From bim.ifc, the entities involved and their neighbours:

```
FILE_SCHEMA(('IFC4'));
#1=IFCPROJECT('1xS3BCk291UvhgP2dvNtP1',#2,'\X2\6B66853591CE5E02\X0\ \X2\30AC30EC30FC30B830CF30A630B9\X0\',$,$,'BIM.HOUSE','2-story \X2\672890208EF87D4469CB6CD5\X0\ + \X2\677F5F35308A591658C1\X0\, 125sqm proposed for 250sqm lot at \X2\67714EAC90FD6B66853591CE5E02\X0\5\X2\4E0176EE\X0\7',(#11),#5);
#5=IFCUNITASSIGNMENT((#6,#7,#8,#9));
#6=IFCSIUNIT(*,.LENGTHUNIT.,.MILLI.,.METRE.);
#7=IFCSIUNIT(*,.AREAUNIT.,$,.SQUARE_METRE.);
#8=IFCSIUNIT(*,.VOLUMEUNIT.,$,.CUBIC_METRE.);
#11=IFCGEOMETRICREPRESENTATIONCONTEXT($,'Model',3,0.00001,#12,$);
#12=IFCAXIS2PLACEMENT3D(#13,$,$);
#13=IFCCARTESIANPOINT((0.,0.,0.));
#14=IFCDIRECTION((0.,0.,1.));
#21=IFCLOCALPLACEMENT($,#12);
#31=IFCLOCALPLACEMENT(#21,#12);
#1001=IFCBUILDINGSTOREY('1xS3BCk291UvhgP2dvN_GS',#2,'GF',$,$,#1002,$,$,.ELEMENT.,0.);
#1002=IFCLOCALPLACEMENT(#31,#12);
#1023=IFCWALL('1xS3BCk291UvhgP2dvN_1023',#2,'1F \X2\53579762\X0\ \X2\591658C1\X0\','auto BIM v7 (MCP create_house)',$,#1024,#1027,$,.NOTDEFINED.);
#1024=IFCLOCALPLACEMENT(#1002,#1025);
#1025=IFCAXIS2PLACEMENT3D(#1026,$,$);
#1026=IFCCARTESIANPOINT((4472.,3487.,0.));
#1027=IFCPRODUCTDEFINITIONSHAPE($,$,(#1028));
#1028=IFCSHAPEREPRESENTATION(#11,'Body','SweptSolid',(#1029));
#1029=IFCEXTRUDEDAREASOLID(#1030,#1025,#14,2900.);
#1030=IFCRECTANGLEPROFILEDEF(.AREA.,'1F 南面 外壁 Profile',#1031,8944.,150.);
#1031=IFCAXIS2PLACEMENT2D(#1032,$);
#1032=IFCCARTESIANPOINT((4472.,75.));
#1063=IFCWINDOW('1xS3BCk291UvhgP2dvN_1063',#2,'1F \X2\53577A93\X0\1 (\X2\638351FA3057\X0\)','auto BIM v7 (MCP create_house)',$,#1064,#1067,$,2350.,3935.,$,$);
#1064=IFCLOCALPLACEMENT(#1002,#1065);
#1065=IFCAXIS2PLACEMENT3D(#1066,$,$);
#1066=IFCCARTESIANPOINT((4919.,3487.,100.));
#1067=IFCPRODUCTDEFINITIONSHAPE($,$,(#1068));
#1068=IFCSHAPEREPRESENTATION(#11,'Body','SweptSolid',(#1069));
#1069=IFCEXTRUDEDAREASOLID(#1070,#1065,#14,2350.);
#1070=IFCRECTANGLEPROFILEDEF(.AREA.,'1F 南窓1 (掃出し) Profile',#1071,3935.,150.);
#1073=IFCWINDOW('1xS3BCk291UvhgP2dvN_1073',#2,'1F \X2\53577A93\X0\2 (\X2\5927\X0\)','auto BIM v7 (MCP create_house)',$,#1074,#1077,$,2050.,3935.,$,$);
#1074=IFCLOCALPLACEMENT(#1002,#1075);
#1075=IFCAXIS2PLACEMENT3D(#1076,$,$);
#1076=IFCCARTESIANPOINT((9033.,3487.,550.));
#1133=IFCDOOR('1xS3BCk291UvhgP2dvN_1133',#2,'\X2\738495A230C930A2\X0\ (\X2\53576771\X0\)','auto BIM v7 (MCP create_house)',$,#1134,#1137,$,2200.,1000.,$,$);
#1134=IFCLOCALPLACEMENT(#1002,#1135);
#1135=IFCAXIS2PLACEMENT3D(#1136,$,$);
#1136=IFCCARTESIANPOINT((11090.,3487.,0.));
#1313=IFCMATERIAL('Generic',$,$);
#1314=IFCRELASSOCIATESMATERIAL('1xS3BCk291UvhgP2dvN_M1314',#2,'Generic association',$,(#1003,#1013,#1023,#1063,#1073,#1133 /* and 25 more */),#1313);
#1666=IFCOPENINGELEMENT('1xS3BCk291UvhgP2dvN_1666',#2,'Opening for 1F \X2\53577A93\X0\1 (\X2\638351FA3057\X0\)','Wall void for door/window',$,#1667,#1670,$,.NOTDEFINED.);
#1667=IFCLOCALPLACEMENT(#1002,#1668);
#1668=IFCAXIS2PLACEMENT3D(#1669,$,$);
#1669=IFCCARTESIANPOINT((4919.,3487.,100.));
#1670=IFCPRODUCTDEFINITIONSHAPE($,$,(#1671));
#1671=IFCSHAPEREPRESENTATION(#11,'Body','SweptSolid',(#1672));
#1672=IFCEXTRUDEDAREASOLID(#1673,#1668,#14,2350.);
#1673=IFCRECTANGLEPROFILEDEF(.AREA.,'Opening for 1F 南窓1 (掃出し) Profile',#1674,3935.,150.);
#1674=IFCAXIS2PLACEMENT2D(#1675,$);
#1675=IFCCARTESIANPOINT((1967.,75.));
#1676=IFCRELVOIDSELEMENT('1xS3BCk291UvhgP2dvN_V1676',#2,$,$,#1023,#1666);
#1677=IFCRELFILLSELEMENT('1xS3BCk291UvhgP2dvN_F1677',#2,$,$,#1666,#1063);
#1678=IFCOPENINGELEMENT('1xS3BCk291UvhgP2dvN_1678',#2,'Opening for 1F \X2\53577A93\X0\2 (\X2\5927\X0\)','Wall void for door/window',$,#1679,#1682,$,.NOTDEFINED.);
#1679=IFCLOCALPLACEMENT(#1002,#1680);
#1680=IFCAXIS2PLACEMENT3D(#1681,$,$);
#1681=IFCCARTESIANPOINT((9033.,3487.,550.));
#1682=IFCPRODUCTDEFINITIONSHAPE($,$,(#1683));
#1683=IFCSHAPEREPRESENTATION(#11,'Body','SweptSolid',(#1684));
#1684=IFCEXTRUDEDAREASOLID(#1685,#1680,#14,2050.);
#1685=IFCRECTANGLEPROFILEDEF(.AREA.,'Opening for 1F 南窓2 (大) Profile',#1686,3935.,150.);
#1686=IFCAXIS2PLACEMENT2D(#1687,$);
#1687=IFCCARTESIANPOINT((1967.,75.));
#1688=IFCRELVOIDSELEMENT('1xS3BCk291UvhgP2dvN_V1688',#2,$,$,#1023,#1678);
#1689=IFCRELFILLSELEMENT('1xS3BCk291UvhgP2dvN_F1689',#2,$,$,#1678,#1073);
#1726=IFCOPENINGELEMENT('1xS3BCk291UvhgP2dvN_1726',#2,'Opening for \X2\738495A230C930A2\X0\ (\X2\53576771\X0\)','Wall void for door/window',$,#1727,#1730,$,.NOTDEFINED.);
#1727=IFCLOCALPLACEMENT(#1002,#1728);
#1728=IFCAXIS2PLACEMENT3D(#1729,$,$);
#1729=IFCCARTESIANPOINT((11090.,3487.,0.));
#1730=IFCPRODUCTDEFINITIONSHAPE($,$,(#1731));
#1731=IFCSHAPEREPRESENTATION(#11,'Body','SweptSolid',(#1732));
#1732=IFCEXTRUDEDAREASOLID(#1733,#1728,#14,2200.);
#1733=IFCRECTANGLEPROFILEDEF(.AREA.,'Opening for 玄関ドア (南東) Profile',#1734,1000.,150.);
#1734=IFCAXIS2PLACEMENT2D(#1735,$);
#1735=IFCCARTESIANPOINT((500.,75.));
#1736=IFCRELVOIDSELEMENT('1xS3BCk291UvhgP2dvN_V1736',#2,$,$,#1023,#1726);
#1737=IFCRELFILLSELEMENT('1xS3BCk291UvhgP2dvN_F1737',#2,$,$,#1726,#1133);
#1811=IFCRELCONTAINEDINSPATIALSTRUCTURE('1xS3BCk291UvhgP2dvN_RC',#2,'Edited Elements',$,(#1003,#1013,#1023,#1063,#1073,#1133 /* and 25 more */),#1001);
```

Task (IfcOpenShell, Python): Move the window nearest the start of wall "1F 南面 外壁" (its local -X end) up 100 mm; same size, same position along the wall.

```python
import numpy as np
import ifcopenshell
import ifcopenshell.api.geometry
import ifcopenshell.util.placement
import ifcopenshell.util.unit

model = ifcopenshell.open("bim.ifc")
unit_scale = ifcopenshell.util.unit.calculate_unit_scale(model)

window = model.by_guid("1xS3BCk291UvhgP2dvN_1063")
opening = window.FillsVoids[0].RelatingOpeningElement
dz = 0.1 / unit_scale

shift = np.array([0.0, 0.0, dz])
# The window is not placed relative to its opening, so move both.
for product in (opening, window):
    matrix = ifcopenshell.util.placement.get_local_placement(product.ObjectPlacement)
    matrix[:3, 3] += shift
    ifcopenshell.api.geometry.edit_object_placement(model, product=product, matrix=matrix, is_si=False)

print(f"moved by {dz * unit_scale:+.3f} m")

model.write("bim_edited.ifc")
```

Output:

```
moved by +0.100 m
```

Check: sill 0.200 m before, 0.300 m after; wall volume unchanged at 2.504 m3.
